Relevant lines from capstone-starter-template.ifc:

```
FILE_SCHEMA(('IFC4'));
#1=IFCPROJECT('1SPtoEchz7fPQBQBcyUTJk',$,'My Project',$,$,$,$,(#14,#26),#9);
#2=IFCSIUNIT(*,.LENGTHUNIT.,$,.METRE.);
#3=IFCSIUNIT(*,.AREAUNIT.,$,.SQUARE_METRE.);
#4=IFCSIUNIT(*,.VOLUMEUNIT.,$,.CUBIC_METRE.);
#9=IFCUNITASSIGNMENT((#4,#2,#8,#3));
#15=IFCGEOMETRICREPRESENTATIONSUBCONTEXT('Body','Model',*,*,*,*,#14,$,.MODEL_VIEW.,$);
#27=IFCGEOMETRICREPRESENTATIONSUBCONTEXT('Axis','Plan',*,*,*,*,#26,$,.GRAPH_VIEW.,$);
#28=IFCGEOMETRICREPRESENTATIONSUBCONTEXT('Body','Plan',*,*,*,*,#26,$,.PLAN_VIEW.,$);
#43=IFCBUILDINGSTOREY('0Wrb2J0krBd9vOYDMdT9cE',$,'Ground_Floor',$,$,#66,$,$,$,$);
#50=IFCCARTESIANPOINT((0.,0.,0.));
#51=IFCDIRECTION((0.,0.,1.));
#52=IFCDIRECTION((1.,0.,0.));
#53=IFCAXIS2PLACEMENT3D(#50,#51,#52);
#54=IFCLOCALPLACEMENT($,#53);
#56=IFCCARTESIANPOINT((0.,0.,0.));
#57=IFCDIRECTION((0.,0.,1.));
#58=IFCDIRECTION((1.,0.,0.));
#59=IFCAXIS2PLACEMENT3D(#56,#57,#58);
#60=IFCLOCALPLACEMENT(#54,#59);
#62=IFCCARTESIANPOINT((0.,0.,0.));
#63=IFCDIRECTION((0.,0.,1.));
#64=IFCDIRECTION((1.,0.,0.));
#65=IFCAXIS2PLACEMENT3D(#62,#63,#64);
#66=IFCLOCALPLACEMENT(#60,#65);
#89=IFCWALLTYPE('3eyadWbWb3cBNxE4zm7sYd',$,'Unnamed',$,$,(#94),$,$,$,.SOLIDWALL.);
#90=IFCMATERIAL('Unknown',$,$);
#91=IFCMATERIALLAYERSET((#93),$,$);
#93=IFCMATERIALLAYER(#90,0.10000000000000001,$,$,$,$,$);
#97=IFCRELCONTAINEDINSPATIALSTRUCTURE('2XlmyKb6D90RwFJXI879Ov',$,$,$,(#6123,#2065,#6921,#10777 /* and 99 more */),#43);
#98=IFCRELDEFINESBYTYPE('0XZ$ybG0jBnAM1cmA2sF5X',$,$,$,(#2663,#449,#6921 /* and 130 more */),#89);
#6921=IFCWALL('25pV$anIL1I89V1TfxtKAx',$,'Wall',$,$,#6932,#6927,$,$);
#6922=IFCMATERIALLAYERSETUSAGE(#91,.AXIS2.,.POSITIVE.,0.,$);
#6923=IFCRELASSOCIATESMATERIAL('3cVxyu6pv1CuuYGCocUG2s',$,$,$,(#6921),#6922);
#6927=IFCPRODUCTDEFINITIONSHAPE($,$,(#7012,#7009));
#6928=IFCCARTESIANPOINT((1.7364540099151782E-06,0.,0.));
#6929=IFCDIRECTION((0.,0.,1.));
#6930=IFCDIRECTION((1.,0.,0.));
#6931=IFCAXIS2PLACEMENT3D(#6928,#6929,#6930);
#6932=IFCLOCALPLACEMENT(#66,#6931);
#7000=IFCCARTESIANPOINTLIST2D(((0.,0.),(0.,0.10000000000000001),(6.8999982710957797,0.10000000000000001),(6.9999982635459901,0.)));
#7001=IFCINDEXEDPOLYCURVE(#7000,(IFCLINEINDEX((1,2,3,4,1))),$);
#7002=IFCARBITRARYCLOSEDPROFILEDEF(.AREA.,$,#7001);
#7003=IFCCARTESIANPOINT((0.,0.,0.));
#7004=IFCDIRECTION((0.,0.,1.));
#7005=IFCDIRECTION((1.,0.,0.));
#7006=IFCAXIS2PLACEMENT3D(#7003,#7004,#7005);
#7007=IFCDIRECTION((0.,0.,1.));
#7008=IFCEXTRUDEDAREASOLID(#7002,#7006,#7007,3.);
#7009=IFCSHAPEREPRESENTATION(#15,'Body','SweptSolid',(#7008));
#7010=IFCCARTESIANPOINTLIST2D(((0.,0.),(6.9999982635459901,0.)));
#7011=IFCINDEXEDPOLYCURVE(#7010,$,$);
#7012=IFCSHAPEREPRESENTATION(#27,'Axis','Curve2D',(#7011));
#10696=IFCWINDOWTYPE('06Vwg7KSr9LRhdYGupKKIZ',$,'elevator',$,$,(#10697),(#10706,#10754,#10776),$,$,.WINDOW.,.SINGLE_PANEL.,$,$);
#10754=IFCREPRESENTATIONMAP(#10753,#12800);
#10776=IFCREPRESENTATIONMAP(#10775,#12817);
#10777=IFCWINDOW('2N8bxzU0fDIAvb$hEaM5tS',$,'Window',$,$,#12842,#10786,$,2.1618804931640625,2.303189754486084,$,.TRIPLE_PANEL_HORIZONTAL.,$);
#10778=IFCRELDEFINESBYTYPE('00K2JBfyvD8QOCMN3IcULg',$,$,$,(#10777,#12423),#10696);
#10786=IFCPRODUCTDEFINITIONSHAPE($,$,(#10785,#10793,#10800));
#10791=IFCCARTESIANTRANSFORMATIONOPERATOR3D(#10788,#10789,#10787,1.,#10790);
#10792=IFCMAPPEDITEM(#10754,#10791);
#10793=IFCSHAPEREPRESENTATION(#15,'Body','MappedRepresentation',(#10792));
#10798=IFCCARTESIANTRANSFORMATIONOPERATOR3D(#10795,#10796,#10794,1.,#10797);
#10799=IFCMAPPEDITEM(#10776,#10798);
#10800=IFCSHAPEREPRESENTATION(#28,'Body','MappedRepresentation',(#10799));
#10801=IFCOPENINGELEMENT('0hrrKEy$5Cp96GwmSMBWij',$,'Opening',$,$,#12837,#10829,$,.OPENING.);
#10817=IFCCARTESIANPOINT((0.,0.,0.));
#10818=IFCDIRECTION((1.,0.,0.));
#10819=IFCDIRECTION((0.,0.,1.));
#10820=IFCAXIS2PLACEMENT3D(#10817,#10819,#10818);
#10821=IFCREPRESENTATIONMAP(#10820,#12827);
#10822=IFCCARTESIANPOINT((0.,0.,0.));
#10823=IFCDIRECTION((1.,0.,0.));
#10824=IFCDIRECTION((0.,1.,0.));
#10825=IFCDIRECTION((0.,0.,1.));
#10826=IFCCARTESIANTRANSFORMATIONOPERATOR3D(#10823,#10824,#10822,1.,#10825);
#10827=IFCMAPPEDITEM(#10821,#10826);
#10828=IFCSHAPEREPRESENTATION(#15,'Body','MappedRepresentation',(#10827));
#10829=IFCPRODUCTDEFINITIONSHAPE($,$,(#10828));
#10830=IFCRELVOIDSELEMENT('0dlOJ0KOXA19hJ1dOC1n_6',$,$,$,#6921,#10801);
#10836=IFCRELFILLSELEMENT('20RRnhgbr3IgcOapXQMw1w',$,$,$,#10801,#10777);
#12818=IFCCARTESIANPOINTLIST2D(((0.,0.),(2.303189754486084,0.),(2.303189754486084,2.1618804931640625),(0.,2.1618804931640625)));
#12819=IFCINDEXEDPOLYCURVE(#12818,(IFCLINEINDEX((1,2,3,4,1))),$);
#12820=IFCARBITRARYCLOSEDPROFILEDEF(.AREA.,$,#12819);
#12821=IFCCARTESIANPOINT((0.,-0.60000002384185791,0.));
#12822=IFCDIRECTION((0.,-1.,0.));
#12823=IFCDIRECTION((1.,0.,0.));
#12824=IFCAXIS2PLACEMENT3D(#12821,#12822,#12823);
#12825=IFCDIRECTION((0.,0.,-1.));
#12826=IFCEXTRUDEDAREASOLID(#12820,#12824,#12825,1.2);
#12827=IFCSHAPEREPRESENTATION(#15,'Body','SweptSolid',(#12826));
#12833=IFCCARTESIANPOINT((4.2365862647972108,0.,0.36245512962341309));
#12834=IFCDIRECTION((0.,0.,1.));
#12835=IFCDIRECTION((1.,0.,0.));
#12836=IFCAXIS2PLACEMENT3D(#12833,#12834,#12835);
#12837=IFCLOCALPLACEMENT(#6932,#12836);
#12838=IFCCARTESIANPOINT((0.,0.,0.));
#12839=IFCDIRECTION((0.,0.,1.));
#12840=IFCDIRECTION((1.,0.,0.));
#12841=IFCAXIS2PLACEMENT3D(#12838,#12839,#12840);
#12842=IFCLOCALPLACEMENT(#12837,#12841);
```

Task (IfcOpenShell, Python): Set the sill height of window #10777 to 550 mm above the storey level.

```python
import numpy as np
import ifcopenshell
import ifcopenshell.api.geometry
import ifcopenshell.geom
import ifcopenshell.util.element
import ifcopenshell.util.placement
import ifcopenshell.util.shape
import ifcopenshell.util.unit

model = ifcopenshell.open("capstone-starter-template.ifc")
unit_scale = ifcopenshell.util.unit.calculate_unit_scale(model)

window = model.by_guid("2N8bxzU0fDIAvb$hEaM5tS")
opening = window.FillsVoids[0].RelatingOpeningElement
storey = ifcopenshell.util.element.get_container(window, ifc_class="IfcBuildingStorey")
level = ifcopenshell.util.placement.get_local_placement(storey.ObjectPlacement)[2, 3]

# The opening's origin need not be at the sill, so measure its lowest point.
shape = ifcopenshell.geom.create_shape(ifcopenshell.geom.settings(), opening)
bottom = ifcopenshell.util.shape.get_shape_bottom_elevation(shape, shape.geometry) / unit_scale
dz = level + 0.55 / unit_scale - bottom

shift = np.array([0.0, 0.0, dz])
# The window is placed relative to its opening, so it follows when the opening moves.
matrix = ifcopenshell.util.placement.get_local_placement(opening.ObjectPlacement)
matrix[:3, 3] += shift
ifcopenshell.api.geometry.edit_object_placement(
    model, product=opening, matrix=matrix, is_si=False, should_transform_children=True
)

print(f"moved by {dz * unit_scale:+.3f} m")

model.write("capstone-starter-template_v2.ifc")
```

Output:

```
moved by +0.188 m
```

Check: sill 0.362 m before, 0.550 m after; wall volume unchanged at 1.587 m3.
